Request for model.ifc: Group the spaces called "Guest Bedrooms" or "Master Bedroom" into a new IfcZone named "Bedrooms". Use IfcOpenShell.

First a look at what the model holds.

```python
import ifcopenshell

model = ifcopenshell.open("model.ifc")
print(model.schema)
seen = {}
for space in model.by_type("IfcSpace"):
    seen[space.Name] = seen.get(space.Name, 0) + 1
for name, count in sorted(seen.items(), key=str):
    print(count, "x", name)
print("zones:", [z.Name for z in model.by_type("IfcZone")][:20])
```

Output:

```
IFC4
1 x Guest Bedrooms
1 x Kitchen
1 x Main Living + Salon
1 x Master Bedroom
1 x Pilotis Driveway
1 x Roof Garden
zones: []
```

```python
import ifcopenshell
import ifcopenshell.api.group
import ifcopenshell.api.root

model = ifcopenshell.open("model.ifc")

names = {"Guest Bedrooms", "Master Bedroom"}
spaces = [s for s in model.by_type("IfcSpace") if s.Name in names]

zone = ifcopenshell.api.root.create_entity(model, ifc_class="IfcZone", name="Bedrooms")
ifcopenshell.api.group.assign_group(model, products=spaces, group=zone)
print(len(spaces), "spaces in", zone.Name)

model.write("model_rev.ifc")
```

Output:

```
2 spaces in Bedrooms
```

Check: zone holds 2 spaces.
